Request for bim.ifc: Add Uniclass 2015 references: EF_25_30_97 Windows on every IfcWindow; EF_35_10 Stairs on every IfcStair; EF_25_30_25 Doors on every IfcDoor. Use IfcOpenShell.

First a look at what the model holds.

```python
import ifcopenshell

model = ifcopenshell.open("bim.ifc")
print(model.schema)
print("classifications:", [c.Name for c in model.by_type("IfcClassification")])
for ifc_class in ("IfcDoor", "IfcRoof", "IfcStair", "IfcWall", "IfcWindow"):
    print(ifc_class, len(model.by_type(ifc_class)))
```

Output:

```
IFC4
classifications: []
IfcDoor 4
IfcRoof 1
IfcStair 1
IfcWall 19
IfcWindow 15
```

```python
import ifcopenshell
import ifcopenshell.api.classification

model = ifcopenshell.open("bim.ifc")

system = ifcopenshell.api.classification.add_classification(model, classification="Uniclass 2015")

codes = {
    "IfcWindow": ("EF_25_30_97", "Windows"),
    "IfcStair": ("EF_35_10", "Stairs"),
    "IfcDoor": ("EF_25_30_25", "Doors"),
}
for ifc_class, (code, name) in codes.items():
    products = model.by_type(ifc_class)
    ifcopenshell.api.classification.add_reference(
        model, products=products, classification=system, identification=code, name=name
    )
    print(code, len(products))

model.write("bim_edited.ifc")
```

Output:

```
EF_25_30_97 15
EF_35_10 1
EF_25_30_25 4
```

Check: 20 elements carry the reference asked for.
